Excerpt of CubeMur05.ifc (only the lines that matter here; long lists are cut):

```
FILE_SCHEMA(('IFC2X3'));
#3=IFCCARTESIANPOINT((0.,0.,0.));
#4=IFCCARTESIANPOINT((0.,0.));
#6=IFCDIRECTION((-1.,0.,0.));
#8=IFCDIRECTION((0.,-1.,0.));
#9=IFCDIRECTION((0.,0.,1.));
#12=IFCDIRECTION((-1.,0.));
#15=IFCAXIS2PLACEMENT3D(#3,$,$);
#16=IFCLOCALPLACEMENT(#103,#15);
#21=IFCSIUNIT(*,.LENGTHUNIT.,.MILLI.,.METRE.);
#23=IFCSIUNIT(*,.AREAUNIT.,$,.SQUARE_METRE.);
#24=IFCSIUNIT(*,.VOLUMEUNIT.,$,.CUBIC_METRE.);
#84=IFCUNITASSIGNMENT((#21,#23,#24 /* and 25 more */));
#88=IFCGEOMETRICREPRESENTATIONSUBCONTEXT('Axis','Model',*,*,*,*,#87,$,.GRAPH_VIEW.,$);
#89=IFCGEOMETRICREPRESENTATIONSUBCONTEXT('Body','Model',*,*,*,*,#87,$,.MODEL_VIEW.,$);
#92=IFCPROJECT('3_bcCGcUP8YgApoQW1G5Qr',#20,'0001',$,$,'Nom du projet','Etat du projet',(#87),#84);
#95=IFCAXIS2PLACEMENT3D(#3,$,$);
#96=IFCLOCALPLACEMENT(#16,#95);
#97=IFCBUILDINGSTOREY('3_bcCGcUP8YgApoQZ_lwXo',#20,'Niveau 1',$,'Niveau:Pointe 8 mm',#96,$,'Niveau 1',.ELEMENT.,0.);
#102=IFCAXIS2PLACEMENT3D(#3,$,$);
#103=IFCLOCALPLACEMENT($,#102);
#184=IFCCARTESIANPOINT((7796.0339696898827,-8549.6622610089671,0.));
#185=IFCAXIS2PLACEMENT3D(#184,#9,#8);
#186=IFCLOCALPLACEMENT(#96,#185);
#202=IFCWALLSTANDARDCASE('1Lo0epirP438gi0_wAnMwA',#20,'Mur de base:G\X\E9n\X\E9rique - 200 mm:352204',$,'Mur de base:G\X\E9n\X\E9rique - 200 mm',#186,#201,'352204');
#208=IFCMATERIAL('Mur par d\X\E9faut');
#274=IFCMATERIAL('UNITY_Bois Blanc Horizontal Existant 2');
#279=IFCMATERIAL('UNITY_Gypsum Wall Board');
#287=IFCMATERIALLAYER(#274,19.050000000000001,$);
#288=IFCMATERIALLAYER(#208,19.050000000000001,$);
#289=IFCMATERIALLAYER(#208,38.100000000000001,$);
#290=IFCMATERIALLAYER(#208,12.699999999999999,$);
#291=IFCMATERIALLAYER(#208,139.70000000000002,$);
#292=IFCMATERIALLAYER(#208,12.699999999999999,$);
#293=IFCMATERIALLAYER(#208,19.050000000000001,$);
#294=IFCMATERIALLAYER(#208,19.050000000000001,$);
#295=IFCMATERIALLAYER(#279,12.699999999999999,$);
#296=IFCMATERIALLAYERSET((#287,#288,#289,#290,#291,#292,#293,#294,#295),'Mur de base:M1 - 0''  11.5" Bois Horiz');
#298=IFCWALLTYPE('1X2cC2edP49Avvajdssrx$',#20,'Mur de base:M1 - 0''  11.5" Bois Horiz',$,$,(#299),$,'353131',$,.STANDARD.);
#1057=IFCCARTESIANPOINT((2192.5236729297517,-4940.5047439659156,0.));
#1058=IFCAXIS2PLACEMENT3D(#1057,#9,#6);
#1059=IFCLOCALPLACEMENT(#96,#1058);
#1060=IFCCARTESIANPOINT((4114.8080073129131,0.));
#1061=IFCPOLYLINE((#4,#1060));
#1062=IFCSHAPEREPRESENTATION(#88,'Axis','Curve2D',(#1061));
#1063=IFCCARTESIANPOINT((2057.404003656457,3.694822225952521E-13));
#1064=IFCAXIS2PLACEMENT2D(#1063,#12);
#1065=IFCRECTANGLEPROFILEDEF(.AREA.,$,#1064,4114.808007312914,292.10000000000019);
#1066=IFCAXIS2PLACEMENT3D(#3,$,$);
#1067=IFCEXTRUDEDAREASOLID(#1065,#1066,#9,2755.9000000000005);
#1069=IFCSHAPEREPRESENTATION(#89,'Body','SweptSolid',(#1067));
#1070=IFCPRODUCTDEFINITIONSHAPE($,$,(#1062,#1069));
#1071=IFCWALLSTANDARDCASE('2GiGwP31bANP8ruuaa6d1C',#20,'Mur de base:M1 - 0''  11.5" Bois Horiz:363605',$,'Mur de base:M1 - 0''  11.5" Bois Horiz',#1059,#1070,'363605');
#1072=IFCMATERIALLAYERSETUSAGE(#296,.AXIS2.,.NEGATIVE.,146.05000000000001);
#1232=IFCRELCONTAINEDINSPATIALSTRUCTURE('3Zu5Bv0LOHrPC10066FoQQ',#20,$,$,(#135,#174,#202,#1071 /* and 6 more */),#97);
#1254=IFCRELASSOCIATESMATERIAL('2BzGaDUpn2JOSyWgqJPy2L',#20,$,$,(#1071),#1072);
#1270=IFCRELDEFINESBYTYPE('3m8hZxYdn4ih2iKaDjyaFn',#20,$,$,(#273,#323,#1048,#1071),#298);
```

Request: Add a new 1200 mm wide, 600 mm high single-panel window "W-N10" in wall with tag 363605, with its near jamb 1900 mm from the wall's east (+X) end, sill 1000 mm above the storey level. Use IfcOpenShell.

```python
import numpy as np
import ifcopenshell
import ifcopenshell.api.feature
import ifcopenshell.api.geometry
import ifcopenshell.api.root
import ifcopenshell.api.spatial
import ifcopenshell.api.type
import ifcopenshell.geom
import ifcopenshell.util.element
import ifcopenshell.util.placement
import ifcopenshell.util.representation
import ifcopenshell.util.shape
import ifcopenshell.util.unit

model = ifcopenshell.open("CubeMur05.ifc")
unit_scale = ifcopenshell.util.unit.calculate_unit_scale(model)
settings = ifcopenshell.geom.settings()


def volume(element):
    """Net volume in cubic metres, openings subtracted."""
    shape = ifcopenshell.geom.create_shape(settings, element)
    return ifcopenshell.util.shape.get_volume(shape.geometry)


wall = model.by_id(1071)
storey = ifcopenshell.util.element.get_container(wall, ifc_class="IfcBuildingStorey")
context = ifcopenshell.util.representation.get_context(model, "Model", "Body", "MODEL_VIEW")
before = volume(wall)

width, height, from_end, sill = 1.2, 0.6, 1.9, 1  # metres

# The wall runs along its own X axis, and the end named is its -X end.
wall_shape = ifcopenshell.geom.create_shape(settings, wall)
x, y, z = ifcopenshell.util.shape.get_vertices(wall_shape.geometry).T
start = x.min() + from_end
face, thickness = float(y.min()), float(y.max() - y.min())
wall_matrix = ifcopenshell.util.placement.get_local_placement(wall.ObjectPlacement)
level = ifcopenshell.util.placement.get_local_placement(storey.ObjectPlacement)[2, 3]


def in_wall(x, y):
    """Placement at x, y metres in the wall's axes, at sill height."""
    matrix = wall_matrix.copy()
    matrix[:, 3] = wall_matrix @ np.array([x / unit_scale, y / unit_scale, 0.0, 1.0])
    matrix[2, 3] = level + sill / unit_scale
    return matrix


# Opening: a box that overshoots both wall faces by 50 mm.
opening = ifcopenshell.api.root.create_entity(model, ifc_class="IfcOpeningElement")
box = ifcopenshell.api.geometry.add_wall_representation(
    model, context=context, length=width, height=height, thickness=thickness + 0.1
)
ifcopenshell.api.geometry.assign_representation(model, product=opening, representation=box)
ifcopenshell.api.geometry.edit_object_placement(model, product=opening, matrix=in_wall(start, face - 0.05), is_si=False)
ifcopenshell.api.feature.add_feature(model, feature=opening, element=wall)

window = ifcopenshell.api.root.create_entity(model, ifc_class="IfcWindow", name="W-N10")
window.OverallWidth, window.OverallHeight = width / unit_scale, height / unit_scale
body = ifcopenshell.api.geometry.add_window_representation(
    model,
    context=context,
    overall_width=window.OverallWidth,
    overall_height=window.OverallHeight,
    partition_type="SINGLE_PANEL",
)
ifcopenshell.api.geometry.assign_representation(model, product=window, representation=body)
ifcopenshell.api.spatial.assign_container(model, products=[window], relating_structure=storey)
fills = ifcopenshell.api.feature.add_filling(model, opening=opening, element=window)
fills.OwnerHistory = window.OwnerHistory  # required in IFC2X3

# IFC2X3 keeps the operation on the window style.
style = ifcopenshell.api.root.create_entity(model, ifc_class="IfcWindowStyle", name="W-N10")
style.OperationType, style.ConstructionType = "SINGLE_PANEL", "NOTDEFINED"
style.ParameterTakesPrecedence = style.Sizeable = False
ifcopenshell.api.type.assign_type(model, related_objects=[window], relating_type=style)

# Centre the window in the wall's thickness.
ifcopenshell.api.geometry.edit_object_placement(model, product=window, matrix=in_wall(start, face), is_si=False)
window_shape = ifcopenshell.geom.create_shape(settings, window)
depth = ifcopenshell.util.shape.get_vertices(window_shape.geometry)[:, 1]
offset = face + thickness / 2 - (depth.min() + depth.max()) / 2
ifcopenshell.api.geometry.edit_object_placement(model, product=window, matrix=in_wall(start, offset), is_si=False)

after = volume(wall)

print(f"wall volume {before:.3f} -> {after:.3f} m3")

model.write("CubeMur05-out.ifc")
```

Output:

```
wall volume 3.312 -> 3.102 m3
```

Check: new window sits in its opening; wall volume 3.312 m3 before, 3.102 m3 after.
